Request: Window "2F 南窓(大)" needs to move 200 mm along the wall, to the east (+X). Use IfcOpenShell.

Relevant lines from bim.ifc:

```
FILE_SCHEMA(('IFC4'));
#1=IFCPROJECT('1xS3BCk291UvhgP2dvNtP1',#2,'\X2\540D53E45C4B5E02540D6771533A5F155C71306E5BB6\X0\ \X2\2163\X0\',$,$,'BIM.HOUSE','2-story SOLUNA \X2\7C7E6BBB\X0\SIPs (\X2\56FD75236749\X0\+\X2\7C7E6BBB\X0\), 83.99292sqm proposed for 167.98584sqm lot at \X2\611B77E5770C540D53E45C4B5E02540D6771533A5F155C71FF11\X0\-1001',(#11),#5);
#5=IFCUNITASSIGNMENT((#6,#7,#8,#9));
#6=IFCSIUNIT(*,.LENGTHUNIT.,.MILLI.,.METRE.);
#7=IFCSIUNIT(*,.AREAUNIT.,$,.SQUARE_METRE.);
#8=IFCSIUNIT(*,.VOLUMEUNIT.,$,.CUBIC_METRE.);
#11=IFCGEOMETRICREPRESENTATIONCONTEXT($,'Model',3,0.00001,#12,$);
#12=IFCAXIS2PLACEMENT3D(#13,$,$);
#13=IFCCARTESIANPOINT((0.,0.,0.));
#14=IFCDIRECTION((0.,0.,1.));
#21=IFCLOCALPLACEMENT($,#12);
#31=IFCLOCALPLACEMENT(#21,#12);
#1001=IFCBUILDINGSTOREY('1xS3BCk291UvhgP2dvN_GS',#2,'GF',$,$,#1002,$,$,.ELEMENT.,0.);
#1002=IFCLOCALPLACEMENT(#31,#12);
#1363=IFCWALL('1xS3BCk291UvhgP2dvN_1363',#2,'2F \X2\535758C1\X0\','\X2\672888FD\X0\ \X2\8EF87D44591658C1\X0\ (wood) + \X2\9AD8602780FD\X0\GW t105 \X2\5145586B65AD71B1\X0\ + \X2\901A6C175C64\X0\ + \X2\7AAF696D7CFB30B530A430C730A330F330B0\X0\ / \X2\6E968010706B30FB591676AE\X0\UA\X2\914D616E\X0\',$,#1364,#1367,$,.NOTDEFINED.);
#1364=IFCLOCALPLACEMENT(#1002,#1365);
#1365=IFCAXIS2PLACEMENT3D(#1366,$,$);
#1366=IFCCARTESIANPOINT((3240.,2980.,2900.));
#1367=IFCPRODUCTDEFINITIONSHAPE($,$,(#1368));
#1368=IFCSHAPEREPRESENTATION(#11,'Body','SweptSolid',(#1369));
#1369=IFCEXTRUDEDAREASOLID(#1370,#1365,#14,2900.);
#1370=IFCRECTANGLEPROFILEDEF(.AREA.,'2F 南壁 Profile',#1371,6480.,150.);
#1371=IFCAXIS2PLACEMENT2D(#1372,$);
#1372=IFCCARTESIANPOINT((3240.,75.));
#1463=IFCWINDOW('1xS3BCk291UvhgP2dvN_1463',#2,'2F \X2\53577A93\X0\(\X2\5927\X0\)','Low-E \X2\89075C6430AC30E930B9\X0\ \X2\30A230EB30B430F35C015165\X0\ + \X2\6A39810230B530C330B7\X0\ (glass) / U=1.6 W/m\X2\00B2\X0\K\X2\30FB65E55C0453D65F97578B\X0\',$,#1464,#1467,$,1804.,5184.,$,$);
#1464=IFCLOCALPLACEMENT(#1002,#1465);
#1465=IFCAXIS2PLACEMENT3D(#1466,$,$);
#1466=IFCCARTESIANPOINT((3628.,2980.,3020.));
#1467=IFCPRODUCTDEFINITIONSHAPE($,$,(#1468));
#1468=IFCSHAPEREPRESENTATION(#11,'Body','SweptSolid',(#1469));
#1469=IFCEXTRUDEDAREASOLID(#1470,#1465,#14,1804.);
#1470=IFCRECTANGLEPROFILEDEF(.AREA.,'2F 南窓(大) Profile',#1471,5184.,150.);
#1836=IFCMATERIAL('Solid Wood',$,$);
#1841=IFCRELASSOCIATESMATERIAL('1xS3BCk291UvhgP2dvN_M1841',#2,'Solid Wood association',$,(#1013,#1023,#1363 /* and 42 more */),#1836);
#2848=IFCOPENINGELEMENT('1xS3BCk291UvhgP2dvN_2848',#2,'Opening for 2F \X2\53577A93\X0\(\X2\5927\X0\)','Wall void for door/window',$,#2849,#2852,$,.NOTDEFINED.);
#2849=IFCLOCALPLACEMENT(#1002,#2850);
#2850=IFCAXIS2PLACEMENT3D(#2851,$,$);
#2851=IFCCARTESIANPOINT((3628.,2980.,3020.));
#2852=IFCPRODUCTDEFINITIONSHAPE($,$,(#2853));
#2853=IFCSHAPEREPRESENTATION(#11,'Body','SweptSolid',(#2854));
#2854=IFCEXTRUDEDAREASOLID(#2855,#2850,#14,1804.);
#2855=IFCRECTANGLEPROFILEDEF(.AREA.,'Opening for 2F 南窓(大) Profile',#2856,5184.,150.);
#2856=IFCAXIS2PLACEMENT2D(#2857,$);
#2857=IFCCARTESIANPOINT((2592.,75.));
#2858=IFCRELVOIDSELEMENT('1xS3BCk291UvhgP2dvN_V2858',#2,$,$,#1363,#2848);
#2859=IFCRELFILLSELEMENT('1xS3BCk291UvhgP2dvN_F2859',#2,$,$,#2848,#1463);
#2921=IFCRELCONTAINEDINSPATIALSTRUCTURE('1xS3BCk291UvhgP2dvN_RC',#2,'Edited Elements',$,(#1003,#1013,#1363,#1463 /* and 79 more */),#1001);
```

```python
import ifcopenshell
import ifcopenshell.api.geometry
import ifcopenshell.util.placement
import ifcopenshell.util.unit

model = ifcopenshell.open("bim.ifc")
unit_scale = ifcopenshell.util.unit.calculate_unit_scale(model)

window = model.by_guid("1xS3BCk291UvhgP2dvN_1463")
opening = window.FillsVoids[0].RelatingOpeningElement
wall = opening.VoidsElements[0].RelatingBuildingElement

wall_matrix = ifcopenshell.util.placement.get_local_placement(wall.ObjectPlacement)
shift = wall_matrix[:3, 0] * 0.2 / unit_scale
before = ifcopenshell.util.placement.get_local_placement(window.ObjectPlacement)[:3, 3].copy()

# The window is not placed relative to its opening, so move both.
for product in (opening, window):
    matrix = ifcopenshell.util.placement.get_local_placement(product.ObjectPlacement)
    matrix[:3, 3] += shift
    ifcopenshell.api.geometry.edit_object_placement(model, product=product, matrix=matrix, is_si=False)

after = ifcopenshell.util.placement.get_local_placement(window.ObjectPlacement)[:3, 3]
print("window moved by", (after - before).round(3) + 0.0)

model.write("bim_rev.ifc")
```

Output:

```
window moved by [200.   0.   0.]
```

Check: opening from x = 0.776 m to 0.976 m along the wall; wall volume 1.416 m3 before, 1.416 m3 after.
